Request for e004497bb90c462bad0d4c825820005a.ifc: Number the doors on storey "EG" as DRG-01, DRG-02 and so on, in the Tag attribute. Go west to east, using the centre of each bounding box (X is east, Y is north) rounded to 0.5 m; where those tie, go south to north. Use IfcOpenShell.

First a look at what the model holds.

```python
import ifcopenshell
import ifcopenshell.util.element
import ifcopenshell.util.placement

model = ifcopenshell.open("e004497bb90c462bad0d4c825820005a.ifc")
print(model.schema)
storey = next(s for s in model.by_type("IfcBuildingStorey") if s.Name == "EG")
doors = [e for e in ifcopenshell.util.element.get_decomposition(storey) if e.is_a("IfcDoor")]
for e in sorted(doors, key=lambda e: e.id()):
    origin = ifcopenshell.util.placement.get_local_placement(e.ObjectPlacement)[:3, 3]
    print(e.id(), e.Tag, e.Name, origin.round(2) + 0.0, sep=" | ")
```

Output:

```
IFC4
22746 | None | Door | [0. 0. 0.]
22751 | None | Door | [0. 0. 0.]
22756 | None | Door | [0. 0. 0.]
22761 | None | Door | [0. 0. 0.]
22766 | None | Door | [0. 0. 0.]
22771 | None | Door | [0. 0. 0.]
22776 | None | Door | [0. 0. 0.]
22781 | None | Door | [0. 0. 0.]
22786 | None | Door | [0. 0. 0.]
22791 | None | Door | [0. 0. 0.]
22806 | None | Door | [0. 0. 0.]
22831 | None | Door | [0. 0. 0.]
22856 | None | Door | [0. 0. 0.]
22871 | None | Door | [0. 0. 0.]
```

```python
import ifcopenshell
import ifcopenshell.geom
import ifcopenshell.util.element
import ifcopenshell.util.shape

model = ifcopenshell.open("e004497bb90c462bad0d4c825820005a.ifc")
settings = ifcopenshell.geom.settings()
settings.set("use-world-coords", True)


def centre(element):
    shape = ifcopenshell.geom.create_shape(settings, element)
    return ifcopenshell.util.shape.get_bbox_centroid(shape.geometry)


storey = next(s for s in model.by_type("IfcBuildingStorey") if s.Name == "EG")
doors = [e for e in ifcopenshell.util.element.get_decomposition(storey) if e.is_a("IfcDoor")]

# Insertion points can sit at a corner or the storey origin, so sort by the geometry (in metres).
centres = {e: centre(e) for e in doors}
doors.sort(key=lambda e: (round(centres[e][0] / 0.5), centres[e][1]))

for i, e in enumerate(doors, start=1):
    number = f"DRG-{i:02d}"
    e.Tag = number
    print(e.id(), number)

model.write("e004497bb90c462bad0d4c825820005a_rev.ifc")
```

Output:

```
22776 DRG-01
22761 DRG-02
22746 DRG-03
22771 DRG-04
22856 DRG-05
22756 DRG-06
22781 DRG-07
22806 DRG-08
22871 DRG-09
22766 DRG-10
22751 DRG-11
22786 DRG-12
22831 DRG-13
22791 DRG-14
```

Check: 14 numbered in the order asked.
